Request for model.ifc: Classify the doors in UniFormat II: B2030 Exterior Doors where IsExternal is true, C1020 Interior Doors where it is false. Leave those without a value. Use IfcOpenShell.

First a look at what the model holds.

```python
import ifcopenshell
import ifcopenshell.util.element

model = ifcopenshell.open("model.ifc")
print(model.schema)
print("classifications:", [c.Name for c in model.by_type("IfcClassification")])
values = [ifcopenshell.util.element.get_pset(e, "Pset_DoorCommon", "IsExternal") for e in model.by_type("IfcDoor")]
for value in (True, False, None):
    print("IsExternal", value, values.count(value))
```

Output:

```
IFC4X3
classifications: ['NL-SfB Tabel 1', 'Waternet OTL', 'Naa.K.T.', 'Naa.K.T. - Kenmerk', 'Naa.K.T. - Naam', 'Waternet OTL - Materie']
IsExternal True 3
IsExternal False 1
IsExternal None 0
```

```python
import ifcopenshell
import ifcopenshell.api.classification
import ifcopenshell.util.element

model = ifcopenshell.open("model.ifc")

system = ifcopenshell.api.classification.add_classification(model, classification="UniFormat II")

doors = model.by_type("IfcDoor")
external = {e: ifcopenshell.util.element.get_pset(e, "Pset_DoorCommon", "IsExternal") for e in doors}
for flag, code, name in ((True, "B2030", "Exterior Doors"), (False, "C1020", "Interior Doors")):
    products = [e for e in doors if external[e] is flag]
    ifcopenshell.api.classification.add_reference(
        model, products=products, classification=system, identification=code, name=name
    )
    print(code, len(products))

model.write("model_v2.ifc")
```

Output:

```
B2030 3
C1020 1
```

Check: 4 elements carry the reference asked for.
